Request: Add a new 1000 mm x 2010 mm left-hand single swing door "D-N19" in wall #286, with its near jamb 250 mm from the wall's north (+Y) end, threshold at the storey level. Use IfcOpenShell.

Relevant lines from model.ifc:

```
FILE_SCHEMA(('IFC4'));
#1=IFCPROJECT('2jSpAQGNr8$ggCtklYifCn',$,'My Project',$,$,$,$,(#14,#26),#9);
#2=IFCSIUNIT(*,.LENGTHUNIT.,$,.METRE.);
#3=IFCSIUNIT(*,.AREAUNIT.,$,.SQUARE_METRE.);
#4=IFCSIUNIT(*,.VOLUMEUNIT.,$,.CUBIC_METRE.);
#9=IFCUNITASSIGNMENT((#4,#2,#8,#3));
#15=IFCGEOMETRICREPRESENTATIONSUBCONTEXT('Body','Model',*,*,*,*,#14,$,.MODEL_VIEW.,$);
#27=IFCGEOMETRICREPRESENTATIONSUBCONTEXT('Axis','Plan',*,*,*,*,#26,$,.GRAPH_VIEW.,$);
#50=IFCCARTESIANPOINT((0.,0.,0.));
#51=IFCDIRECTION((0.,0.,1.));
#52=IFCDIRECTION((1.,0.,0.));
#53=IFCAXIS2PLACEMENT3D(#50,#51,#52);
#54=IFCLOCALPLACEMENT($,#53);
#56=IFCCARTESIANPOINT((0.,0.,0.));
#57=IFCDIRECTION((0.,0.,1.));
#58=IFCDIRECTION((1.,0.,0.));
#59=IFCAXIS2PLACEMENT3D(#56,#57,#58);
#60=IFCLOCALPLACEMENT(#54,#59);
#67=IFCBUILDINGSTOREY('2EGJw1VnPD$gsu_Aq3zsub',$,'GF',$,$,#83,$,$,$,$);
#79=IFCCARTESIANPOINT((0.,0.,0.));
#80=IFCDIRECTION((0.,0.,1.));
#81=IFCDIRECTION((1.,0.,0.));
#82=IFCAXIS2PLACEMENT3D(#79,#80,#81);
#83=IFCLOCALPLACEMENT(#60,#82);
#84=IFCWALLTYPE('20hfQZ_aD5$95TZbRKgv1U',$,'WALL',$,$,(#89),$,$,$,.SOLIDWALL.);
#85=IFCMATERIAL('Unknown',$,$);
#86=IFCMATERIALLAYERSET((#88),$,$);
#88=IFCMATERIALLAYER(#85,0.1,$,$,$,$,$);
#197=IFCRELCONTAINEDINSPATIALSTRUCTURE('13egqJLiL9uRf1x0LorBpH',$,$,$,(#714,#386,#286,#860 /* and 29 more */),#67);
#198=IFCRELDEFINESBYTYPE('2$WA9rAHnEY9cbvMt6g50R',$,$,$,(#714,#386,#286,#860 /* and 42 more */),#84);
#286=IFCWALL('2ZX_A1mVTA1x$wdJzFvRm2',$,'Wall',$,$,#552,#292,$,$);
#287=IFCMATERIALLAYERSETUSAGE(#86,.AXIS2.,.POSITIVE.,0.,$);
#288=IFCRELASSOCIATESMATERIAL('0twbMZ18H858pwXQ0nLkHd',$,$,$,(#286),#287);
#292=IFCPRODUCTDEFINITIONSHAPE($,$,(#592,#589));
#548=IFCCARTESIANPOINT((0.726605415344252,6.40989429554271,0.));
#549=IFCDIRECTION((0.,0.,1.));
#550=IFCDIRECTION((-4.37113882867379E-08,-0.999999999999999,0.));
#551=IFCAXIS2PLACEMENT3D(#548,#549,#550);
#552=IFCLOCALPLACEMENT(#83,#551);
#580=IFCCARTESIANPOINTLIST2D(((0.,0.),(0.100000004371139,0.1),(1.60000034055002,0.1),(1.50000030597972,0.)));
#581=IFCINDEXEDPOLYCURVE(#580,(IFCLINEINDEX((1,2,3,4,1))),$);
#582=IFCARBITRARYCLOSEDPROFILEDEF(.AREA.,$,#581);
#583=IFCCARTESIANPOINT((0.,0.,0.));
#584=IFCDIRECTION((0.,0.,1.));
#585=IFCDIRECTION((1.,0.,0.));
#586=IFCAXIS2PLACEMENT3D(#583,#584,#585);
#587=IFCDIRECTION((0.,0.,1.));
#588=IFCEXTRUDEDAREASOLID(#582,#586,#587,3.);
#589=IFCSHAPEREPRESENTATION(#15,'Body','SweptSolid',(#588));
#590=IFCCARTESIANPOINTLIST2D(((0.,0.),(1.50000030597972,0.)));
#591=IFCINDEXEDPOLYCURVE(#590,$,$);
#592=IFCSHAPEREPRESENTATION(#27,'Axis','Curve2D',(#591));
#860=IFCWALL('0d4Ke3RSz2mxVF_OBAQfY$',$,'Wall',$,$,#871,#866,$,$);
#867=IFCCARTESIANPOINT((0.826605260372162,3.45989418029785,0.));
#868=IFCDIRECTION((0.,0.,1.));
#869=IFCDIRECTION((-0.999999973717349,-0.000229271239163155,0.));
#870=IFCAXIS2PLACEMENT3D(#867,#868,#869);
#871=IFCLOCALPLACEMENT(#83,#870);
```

```python
import numpy as np
import ifcopenshell
import ifcopenshell.api.feature
import ifcopenshell.api.geometry
import ifcopenshell.api.root
import ifcopenshell.api.spatial
import ifcopenshell.geom
import ifcopenshell.util.element
import ifcopenshell.util.placement
import ifcopenshell.util.representation
import ifcopenshell.util.shape
import ifcopenshell.util.unit

model = ifcopenshell.open("model.ifc")
unit_scale = ifcopenshell.util.unit.calculate_unit_scale(model)
settings = ifcopenshell.geom.settings()


def volume(element):
    """Net volume in cubic metres, openings subtracted."""
    shape = ifcopenshell.geom.create_shape(settings, element)
    return ifcopenshell.util.shape.get_volume(shape.geometry)


wall = model.by_guid("2ZX_A1mVTA1x$wdJzFvRm2")
storey = ifcopenshell.util.element.get_container(wall, ifc_class="IfcBuildingStorey")
context = ifcopenshell.util.representation.get_context(model, "Model", "Body", "MODEL_VIEW")
before = volume(wall)

width, height, from_end, sill = 1, 2.01, 0.25, 0.0  # metres

# The wall runs along its own X axis, and the end named is its -X end.
wall_shape = ifcopenshell.geom.create_shape(settings, wall)
x, y, z = ifcopenshell.util.shape.get_vertices(wall_shape.geometry).T
start = x.min() + from_end
face, thickness = float(y.min()), float(y.max() - y.min())
wall_matrix = ifcopenshell.util.placement.get_local_placement(wall.ObjectPlacement)
level = ifcopenshell.util.placement.get_local_placement(storey.ObjectPlacement)[2, 3]


def in_wall(x, y):
    """Placement at x, y metres in the wall's axes, at sill height."""
    matrix = wall_matrix.copy()
    matrix[:, 3] = wall_matrix @ np.array([x / unit_scale, y / unit_scale, 0.0, 1.0])
    matrix[2, 3] = level + sill / unit_scale
    return matrix


# Opening: a box that overshoots both wall faces by 50 mm.
opening = ifcopenshell.api.root.create_entity(model, ifc_class="IfcOpeningElement", predefined_type="OPENING")
box = ifcopenshell.api.geometry.add_wall_representation(
    model, context=context, length=width, height=height, thickness=thickness + 0.1
)
ifcopenshell.api.geometry.assign_representation(model, product=opening, representation=box)
ifcopenshell.api.geometry.edit_object_placement(model, product=opening, matrix=in_wall(start, face - 0.05), is_si=False)
ifcopenshell.api.feature.add_feature(model, feature=opening, element=wall)

door = ifcopenshell.api.root.create_entity(model, ifc_class="IfcDoor", name="D-N19", predefined_type="DOOR")
door.OverallWidth, door.OverallHeight = width / unit_scale, height / unit_scale
door.OperationType = "SINGLE_SWING_LEFT"
body = ifcopenshell.api.geometry.add_door_representation(
    model,
    context=context,
    overall_width=door.OverallWidth,
    overall_height=door.OverallHeight,
    operation_type="SINGLE_SWING_LEFT",
    lining_properties={"LiningDepth": thickness / unit_scale, "ThresholdDepth": thickness / unit_scale},
)
ifcopenshell.api.geometry.assign_representation(model, product=door, representation=body)
ifcopenshell.api.spatial.assign_container(model, products=[door], relating_structure=storey)
ifcopenshell.api.feature.add_filling(model, opening=opening, element=door)

# The lining spans the wall, so the door starts at the wall face.
ifcopenshell.api.geometry.edit_object_placement(model, product=door, matrix=in_wall(start, face), is_si=False)

after = volume(wall)

print(f"wall volume {before:.3f} -> {after:.3f} m3")

model.write("model_updated.ifc")
```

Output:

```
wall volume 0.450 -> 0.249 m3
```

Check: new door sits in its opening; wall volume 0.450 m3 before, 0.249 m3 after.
